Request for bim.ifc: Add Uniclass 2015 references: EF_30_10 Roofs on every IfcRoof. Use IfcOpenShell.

First a look at what the model holds.

```python
import ifcopenshell

model = ifcopenshell.open("bim.ifc")
print(model.schema)
print("classifications:", [c.Name for c in model.by_type("IfcClassification")])
for ifc_class in ("IfcDoor", "IfcRoof", "IfcStair", "IfcWall", "IfcWindow"):
    print(ifc_class, len(model.by_type(ifc_class)))
```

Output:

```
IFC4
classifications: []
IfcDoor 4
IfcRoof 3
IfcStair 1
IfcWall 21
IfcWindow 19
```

```python
import ifcopenshell
import ifcopenshell.api.classification

model = ifcopenshell.open("bim.ifc")

system = ifcopenshell.api.classification.add_classification(model, classification="Uniclass 2015")

codes = {
    "IfcRoof": ("EF_30_10", "Roofs"),
}
for ifc_class, (code, name) in codes.items():
    products = model.by_type(ifc_class)
    ifcopenshell.api.classification.add_reference(
        model, products=products, classification=system, identification=code, name=name
    )
    print(code, len(products))

model.write("bim_rev.ifc")
```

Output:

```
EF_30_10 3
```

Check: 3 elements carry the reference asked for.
